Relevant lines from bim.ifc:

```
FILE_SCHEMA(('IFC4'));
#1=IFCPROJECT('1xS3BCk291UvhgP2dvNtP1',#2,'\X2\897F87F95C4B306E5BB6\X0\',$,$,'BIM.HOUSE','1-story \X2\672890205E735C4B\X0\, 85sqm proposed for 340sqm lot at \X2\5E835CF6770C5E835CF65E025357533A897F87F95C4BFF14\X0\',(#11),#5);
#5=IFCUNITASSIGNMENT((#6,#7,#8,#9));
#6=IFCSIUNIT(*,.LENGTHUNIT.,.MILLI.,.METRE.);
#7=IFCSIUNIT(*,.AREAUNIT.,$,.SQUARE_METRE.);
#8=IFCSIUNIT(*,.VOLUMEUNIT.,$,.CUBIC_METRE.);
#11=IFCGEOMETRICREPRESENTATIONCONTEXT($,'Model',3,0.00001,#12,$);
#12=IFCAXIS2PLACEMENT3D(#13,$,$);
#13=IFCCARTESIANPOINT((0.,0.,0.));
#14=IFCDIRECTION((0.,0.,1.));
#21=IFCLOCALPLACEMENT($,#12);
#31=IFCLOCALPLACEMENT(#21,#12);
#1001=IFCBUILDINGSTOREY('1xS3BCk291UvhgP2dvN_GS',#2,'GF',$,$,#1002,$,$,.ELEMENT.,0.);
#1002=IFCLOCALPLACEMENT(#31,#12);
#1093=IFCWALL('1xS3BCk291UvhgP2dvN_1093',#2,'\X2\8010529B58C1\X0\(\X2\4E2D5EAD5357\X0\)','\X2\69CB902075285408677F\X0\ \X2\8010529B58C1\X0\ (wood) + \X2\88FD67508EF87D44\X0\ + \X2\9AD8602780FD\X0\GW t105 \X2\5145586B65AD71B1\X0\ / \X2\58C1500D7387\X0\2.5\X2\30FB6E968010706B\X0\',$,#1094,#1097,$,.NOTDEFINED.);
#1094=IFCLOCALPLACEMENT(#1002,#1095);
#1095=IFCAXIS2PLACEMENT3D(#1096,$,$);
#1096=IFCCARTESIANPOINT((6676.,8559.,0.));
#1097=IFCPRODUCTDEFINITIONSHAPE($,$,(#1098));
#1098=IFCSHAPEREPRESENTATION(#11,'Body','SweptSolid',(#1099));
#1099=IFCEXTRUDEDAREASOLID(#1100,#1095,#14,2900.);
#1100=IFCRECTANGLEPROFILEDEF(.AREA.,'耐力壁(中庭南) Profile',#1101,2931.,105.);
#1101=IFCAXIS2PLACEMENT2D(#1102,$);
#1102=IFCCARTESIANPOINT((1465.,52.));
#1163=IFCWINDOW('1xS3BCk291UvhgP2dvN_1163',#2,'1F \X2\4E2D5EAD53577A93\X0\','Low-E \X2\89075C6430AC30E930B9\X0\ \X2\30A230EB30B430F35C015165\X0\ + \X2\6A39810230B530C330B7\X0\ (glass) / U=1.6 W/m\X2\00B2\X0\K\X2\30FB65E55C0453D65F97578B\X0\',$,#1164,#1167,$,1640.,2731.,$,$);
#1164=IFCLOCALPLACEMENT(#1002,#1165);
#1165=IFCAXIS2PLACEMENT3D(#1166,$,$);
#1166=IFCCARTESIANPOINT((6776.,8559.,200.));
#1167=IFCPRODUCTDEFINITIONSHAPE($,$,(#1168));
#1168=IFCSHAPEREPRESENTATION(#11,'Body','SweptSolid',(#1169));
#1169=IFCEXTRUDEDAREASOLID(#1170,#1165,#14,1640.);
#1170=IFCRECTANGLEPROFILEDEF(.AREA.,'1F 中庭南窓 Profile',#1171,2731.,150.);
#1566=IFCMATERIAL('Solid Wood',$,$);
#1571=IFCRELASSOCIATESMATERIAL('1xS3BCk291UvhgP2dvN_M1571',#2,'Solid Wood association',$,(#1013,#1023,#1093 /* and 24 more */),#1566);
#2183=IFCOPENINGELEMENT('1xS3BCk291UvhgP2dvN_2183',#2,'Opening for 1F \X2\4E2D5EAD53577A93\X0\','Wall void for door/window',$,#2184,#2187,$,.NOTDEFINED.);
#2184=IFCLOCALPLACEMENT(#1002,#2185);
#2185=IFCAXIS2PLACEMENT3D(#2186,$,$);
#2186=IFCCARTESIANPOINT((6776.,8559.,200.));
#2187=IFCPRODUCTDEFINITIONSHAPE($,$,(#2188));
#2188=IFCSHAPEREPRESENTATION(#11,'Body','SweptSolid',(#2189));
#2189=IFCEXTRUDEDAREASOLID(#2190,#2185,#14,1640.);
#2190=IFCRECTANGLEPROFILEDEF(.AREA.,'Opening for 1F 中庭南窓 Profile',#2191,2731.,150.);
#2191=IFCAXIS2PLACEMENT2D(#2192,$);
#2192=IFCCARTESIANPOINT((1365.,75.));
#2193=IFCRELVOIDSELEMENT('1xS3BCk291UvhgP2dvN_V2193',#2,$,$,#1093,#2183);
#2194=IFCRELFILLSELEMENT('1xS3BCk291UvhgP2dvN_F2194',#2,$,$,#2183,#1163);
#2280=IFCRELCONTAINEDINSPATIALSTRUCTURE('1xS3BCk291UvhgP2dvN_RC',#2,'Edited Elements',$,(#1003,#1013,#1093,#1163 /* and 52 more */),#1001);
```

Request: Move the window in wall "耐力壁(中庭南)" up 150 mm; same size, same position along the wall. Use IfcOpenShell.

```python
import numpy as np
import ifcopenshell
import ifcopenshell.api.geometry
import ifcopenshell.util.placement
import ifcopenshell.util.unit

model = ifcopenshell.open("bim.ifc")
unit_scale = ifcopenshell.util.unit.calculate_unit_scale(model)

window = model.by_guid("1xS3BCk291UvhgP2dvN_1163")
opening = window.FillsVoids[0].RelatingOpeningElement
dz = 150.0

shift = np.array([0.0, 0.0, dz])
# The window is not placed relative to its opening, so move both.
for product in (opening, window):
    matrix = ifcopenshell.util.placement.get_local_placement(product.ObjectPlacement)
    matrix[:3, 3] += shift
    ifcopenshell.api.geometry.edit_object_placement(model, product=product, matrix=matrix, is_si=False)

print(f"moved by {dz * unit_scale:+.3f} m")

model.write("bim_v2.ifc")
```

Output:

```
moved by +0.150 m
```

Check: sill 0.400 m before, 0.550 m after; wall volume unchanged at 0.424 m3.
